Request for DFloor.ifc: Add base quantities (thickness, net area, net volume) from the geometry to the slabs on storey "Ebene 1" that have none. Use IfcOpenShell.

First a look at what the model holds.

```python
import ifcopenshell
import ifcopenshell.util.element
import ifcopenshell.util.unit

model = ifcopenshell.open("DFloor.ifc")
print(model.schema)
for unit_type in ("LENGTHUNIT", "AREAUNIT", "VOLUMEUNIT"):
    print(unit_type, ifcopenshell.util.unit.calculate_unit_scale(model, unit_type))
storey = next(s for s in model.by_type("IfcBuildingStorey") if s.Name == "Ebene 1")
slabs = [e for e in ifcopenshell.util.element.get_decomposition(storey) if e.is_a("IfcSlab")]
for e in sorted(slabs, key=lambda e: e.id()):
    print(e.id(), e.is_a(), e.Name, list(ifcopenshell.util.element.get_psets(e, qtos_only=True)), sep=" | ")
```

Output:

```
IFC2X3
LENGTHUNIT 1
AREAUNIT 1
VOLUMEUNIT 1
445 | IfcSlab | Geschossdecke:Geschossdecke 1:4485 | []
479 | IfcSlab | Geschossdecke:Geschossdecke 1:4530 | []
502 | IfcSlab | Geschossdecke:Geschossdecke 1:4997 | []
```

```python
import ifcopenshell
import ifcopenshell.api.pset
import ifcopenshell.geom
import ifcopenshell.util.element
import ifcopenshell.util.shape
import ifcopenshell.util.unit

model = ifcopenshell.open("DFloor.ifc")
unit_scale = ifcopenshell.util.unit.calculate_unit_scale(model)
area_scale = ifcopenshell.util.unit.calculate_unit_scale(model, "AREAUNIT")
volume_scale = ifcopenshell.util.unit.calculate_unit_scale(model, "VOLUMEUNIT")
settings = ifcopenshell.geom.settings()

storey = next(s for s in model.by_type("IfcBuildingStorey") if s.Name == "Ebene 1")
slabs = [e for e in ifcopenshell.util.element.get_decomposition(storey) if e.is_a("IfcSlab")]

for e in sorted(slabs, key=lambda e: e.id()):
    if ifcopenshell.util.element.get_psets(e, qtos_only=True, should_inherit=False):
        continue
    # Geometry comes back in metres, in the element's own axes.
    shape = ifcopenshell.geom.create_shape(settings, e)
    values = {
        "Width": ifcopenshell.util.shape.get_z(shape.geometry) / unit_scale,
        "NetArea": ifcopenshell.util.shape.get_footprint_area(shape.geometry) / area_scale,
        "NetVolume": ifcopenshell.util.shape.get_volume(shape.geometry) / volume_scale,
    }
    qto = ifcopenshell.api.pset.add_qto(model, product=e, name="BaseQuantities")
    ifcopenshell.api.pset.edit_qto(model, qto=qto, properties=values)
    print(e.id(), {k: round(v, 3) for k, v in values.items()})

model.write("DFloor_edited.ifc")
```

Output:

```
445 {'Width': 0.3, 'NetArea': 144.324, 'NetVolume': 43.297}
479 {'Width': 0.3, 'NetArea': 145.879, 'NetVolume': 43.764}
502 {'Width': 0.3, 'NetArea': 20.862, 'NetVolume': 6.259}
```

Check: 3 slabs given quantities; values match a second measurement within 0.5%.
